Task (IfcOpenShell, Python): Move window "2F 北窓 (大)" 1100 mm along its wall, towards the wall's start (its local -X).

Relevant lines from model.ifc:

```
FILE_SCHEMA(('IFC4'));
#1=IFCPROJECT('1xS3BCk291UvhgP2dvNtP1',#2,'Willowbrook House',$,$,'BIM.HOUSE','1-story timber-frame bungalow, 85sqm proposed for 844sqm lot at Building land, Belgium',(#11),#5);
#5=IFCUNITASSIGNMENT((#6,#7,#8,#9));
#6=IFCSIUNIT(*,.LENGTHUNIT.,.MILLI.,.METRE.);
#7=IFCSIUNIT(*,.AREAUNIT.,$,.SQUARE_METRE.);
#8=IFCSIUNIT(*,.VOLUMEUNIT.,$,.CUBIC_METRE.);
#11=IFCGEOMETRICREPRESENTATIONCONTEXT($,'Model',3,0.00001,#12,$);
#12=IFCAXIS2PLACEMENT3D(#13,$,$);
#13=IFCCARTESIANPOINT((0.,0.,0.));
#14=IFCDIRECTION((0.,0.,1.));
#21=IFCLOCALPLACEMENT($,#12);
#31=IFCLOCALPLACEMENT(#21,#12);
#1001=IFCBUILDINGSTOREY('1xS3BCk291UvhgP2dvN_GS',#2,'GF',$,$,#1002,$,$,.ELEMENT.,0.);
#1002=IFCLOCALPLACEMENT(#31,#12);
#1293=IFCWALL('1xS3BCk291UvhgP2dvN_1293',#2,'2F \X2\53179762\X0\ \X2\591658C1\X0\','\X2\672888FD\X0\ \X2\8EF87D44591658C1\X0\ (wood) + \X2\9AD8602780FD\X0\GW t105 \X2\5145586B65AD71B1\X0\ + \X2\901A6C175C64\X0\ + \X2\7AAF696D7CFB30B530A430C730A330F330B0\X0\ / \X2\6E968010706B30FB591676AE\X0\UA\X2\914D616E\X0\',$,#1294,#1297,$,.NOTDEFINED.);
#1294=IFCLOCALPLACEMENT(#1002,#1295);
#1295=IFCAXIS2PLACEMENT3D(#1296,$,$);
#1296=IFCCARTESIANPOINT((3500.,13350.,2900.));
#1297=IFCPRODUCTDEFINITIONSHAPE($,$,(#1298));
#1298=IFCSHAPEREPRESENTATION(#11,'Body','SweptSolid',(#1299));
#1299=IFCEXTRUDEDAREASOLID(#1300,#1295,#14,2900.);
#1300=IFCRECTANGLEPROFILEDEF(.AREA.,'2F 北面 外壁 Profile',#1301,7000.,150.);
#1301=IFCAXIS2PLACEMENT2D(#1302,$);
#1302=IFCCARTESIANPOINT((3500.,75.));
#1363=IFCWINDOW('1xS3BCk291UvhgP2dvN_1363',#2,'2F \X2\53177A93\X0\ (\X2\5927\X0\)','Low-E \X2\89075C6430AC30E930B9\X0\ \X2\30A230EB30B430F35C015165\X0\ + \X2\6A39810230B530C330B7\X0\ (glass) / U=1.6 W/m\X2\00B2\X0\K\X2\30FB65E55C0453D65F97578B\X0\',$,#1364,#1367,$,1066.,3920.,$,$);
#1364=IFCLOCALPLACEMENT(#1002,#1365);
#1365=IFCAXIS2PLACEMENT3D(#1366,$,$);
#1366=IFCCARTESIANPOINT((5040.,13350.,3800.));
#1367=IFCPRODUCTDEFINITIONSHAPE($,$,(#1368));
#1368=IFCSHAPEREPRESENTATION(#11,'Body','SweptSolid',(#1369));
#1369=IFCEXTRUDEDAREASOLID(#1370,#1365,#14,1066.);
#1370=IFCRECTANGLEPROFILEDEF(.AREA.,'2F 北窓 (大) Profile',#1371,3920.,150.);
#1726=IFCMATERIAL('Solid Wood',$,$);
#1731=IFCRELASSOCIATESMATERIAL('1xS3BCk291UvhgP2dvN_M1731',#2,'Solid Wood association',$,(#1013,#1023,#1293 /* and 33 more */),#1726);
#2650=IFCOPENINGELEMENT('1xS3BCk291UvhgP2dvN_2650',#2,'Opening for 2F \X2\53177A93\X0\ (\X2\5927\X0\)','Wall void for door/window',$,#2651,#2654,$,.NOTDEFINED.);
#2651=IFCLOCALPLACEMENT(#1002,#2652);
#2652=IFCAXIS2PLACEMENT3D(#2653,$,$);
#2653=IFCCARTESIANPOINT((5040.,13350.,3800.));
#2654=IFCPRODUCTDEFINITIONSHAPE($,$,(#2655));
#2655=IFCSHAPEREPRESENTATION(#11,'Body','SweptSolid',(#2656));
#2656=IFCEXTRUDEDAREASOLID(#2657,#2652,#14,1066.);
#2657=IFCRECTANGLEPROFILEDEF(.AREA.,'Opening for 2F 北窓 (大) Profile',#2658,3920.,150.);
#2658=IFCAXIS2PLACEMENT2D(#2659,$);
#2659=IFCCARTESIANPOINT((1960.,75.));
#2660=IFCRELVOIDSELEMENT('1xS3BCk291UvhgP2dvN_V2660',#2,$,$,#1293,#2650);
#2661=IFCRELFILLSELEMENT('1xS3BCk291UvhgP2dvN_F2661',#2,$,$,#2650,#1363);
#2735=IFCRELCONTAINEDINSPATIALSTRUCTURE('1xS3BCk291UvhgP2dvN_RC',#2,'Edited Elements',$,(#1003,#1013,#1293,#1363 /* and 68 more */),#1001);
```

```python
import ifcopenshell
import ifcopenshell.api.geometry
import ifcopenshell.util.placement

model = ifcopenshell.open("model.ifc")

window = model.by_id(1363)
opening = window.FillsVoids[0].RelatingOpeningElement
wall = opening.VoidsElements[0].RelatingBuildingElement

wall_matrix = ifcopenshell.util.placement.get_local_placement(wall.ObjectPlacement)
shift = wall_matrix[:3, 0] * -1100.0
before = ifcopenshell.util.placement.get_local_placement(window.ObjectPlacement)[:3, 3].copy()

# The window is not placed relative to its opening, so move both.
for product in (opening, window):
    matrix = ifcopenshell.util.placement.get_local_placement(product.ObjectPlacement)
    matrix[:3, 3] += shift
    ifcopenshell.api.geometry.edit_object_placement(model, product=product, matrix=matrix, is_si=False)

after = ifcopenshell.util.placement.get_local_placement(window.ObjectPlacement)[:3, 3]
print("window moved by", (after - before).round(3) + 0.0)

model.write("model_v2.ifc")
```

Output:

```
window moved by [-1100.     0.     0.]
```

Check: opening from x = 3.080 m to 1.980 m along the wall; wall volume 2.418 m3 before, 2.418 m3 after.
